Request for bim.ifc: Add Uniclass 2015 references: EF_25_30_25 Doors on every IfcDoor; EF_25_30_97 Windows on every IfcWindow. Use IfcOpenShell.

First a look at what the model holds.

```python
import ifcopenshell

model = ifcopenshell.open("bim.ifc")
print(model.schema)
print("classifications:", [c.Name for c in model.by_type("IfcClassification")])
for ifc_class in ("IfcDoor", "IfcRoof", "IfcStair", "IfcWall", "IfcWindow"):
    print(ifc_class, len(model.by_type(ifc_class)))
```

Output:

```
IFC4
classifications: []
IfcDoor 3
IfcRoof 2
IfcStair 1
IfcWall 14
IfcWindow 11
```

```python
import ifcopenshell
import ifcopenshell.api.classification

model = ifcopenshell.open("bim.ifc")

system = ifcopenshell.api.classification.add_classification(model, classification="Uniclass 2015")

codes = {
    "IfcDoor": ("EF_25_30_25", "Doors"),
    "IfcWindow": ("EF_25_30_97", "Windows"),
}
for ifc_class, (code, name) in codes.items():
    products = model.by_type(ifc_class)
    ifcopenshell.api.classification.add_reference(
        model, products=products, classification=system, identification=code, name=name
    )
    print(code, len(products))

model.write("bim-out.ifc")
```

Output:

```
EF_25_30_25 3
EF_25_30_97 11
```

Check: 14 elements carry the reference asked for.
